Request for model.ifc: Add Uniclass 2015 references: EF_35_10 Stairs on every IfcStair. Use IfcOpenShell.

First a look at what the model holds.

```python
import ifcopenshell

model = ifcopenshell.open("model.ifc")
print(model.schema)
print("classifications:", [c.Name for c in model.by_type("IfcClassification")])
for ifc_class in ("IfcDoor", "IfcRoof", "IfcStair", "IfcWall", "IfcWindow"):
    print(ifc_class, len(model.by_type(ifc_class)))
```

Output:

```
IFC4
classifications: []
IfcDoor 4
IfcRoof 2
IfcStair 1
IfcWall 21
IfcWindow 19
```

```python
import ifcopenshell
import ifcopenshell.api.classification

model = ifcopenshell.open("model.ifc")

system = ifcopenshell.api.classification.add_classification(model, classification="Uniclass 2015")

codes = {
    "IfcStair": ("EF_35_10", "Stairs"),
}
for ifc_class, (code, name) in codes.items():
    products = model.by_type(ifc_class)
    ifcopenshell.api.classification.add_reference(
        model, products=products, classification=system, identification=code, name=name
    )
    print(code, len(products))

model.write("model_rev.ifc")
```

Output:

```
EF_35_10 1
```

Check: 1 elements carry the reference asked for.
